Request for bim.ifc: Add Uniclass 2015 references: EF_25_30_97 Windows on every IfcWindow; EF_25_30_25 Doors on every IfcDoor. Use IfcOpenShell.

First a look at what the model holds.

```python
import ifcopenshell

model = ifcopenshell.open("bim.ifc")
print(model.schema)
print("classifications:", [c.Name for c in model.by_type("IfcClassification")])
for ifc_class in ("IfcDoor", "IfcRoof", "IfcStair", "IfcWall", "IfcWindow"):
    print(ifc_class, len(model.by_type(ifc_class)))
```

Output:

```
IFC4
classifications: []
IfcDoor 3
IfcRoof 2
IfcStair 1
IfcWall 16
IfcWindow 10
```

```python
import ifcopenshell
import ifcopenshell.api.classification

model = ifcopenshell.open("bim.ifc")

system = ifcopenshell.api.classification.add_classification(model, classification="Uniclass 2015")

codes = {
    "IfcWindow": ("EF_25_30_97", "Windows"),
    "IfcDoor": ("EF_25_30_25", "Doors"),
}
for ifc_class, (code, name) in codes.items():
    products = model.by_type(ifc_class)
    ifcopenshell.api.classification.add_reference(
        model, products=products, classification=system, identification=code, name=name
    )
    print(code, len(products))

model.write("bim_edited.ifc")
```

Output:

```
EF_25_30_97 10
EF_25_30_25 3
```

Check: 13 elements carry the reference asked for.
